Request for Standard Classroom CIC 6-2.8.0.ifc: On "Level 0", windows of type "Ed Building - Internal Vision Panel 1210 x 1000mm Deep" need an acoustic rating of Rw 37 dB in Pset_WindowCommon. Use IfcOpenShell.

First a look at what the model holds.

```python
import ifcopenshell
import ifcopenshell.util.element

model = ifcopenshell.open("Standard Classroom CIC 6-2.8.0.ifc")
print(model.schema)
storey = next(s for s in model.by_type("IfcBuildingStorey") if s.Name == "Level 0")
windows = [e for e in ifcopenshell.util.element.get_decomposition(storey) if e.is_a("IfcWindow")]
seen = {}
for e in windows:
    element_type = ifcopenshell.util.element.get_type(e)
    key = (element_type.Name if element_type != e and element_type else None, ifcopenshell.util.element.get_pset(e, "Pset_WindowCommon", "AcousticRating"))
    seen[key] = seen.get(key, 0) + 1
for (name, value), count in sorted(seen.items(), key=str):
    print(count, "x", name, "|", value)
```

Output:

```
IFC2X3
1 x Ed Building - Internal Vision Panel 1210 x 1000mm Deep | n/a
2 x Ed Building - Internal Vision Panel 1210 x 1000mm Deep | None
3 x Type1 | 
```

```python
import ifcopenshell
import ifcopenshell.api.pset
import ifcopenshell.util.element

model = ifcopenshell.open("Standard Classroom CIC 6-2.8.0.ifc")

storey = next(s for s in model.by_type("IfcBuildingStorey") if s.Name == "Level 0")
windows = [e for e in ifcopenshell.util.element.get_decomposition(storey) if e.is_a("IfcWindow")]

count = 0
for e in windows:
    element_type = ifcopenshell.util.element.get_type(e)
    if element_type in (None, e) or element_type.Name != "Ed Building - Internal Vision Panel 1210 x 1000mm Deep":
        continue
    # add_pset returns the element's existing set when there is one.
    pset = ifcopenshell.api.pset.add_pset(model, product=e, name="Pset_WindowCommon")
    ifcopenshell.api.pset.edit_pset(model, pset=pset, properties={"AcousticRating": "Rw 37 dB"})
    count += 1

print(count, "windows updated")

model.write("Standard Classroom CIC 6-2.8.0-out.ifc")
```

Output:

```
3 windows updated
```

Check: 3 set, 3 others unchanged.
